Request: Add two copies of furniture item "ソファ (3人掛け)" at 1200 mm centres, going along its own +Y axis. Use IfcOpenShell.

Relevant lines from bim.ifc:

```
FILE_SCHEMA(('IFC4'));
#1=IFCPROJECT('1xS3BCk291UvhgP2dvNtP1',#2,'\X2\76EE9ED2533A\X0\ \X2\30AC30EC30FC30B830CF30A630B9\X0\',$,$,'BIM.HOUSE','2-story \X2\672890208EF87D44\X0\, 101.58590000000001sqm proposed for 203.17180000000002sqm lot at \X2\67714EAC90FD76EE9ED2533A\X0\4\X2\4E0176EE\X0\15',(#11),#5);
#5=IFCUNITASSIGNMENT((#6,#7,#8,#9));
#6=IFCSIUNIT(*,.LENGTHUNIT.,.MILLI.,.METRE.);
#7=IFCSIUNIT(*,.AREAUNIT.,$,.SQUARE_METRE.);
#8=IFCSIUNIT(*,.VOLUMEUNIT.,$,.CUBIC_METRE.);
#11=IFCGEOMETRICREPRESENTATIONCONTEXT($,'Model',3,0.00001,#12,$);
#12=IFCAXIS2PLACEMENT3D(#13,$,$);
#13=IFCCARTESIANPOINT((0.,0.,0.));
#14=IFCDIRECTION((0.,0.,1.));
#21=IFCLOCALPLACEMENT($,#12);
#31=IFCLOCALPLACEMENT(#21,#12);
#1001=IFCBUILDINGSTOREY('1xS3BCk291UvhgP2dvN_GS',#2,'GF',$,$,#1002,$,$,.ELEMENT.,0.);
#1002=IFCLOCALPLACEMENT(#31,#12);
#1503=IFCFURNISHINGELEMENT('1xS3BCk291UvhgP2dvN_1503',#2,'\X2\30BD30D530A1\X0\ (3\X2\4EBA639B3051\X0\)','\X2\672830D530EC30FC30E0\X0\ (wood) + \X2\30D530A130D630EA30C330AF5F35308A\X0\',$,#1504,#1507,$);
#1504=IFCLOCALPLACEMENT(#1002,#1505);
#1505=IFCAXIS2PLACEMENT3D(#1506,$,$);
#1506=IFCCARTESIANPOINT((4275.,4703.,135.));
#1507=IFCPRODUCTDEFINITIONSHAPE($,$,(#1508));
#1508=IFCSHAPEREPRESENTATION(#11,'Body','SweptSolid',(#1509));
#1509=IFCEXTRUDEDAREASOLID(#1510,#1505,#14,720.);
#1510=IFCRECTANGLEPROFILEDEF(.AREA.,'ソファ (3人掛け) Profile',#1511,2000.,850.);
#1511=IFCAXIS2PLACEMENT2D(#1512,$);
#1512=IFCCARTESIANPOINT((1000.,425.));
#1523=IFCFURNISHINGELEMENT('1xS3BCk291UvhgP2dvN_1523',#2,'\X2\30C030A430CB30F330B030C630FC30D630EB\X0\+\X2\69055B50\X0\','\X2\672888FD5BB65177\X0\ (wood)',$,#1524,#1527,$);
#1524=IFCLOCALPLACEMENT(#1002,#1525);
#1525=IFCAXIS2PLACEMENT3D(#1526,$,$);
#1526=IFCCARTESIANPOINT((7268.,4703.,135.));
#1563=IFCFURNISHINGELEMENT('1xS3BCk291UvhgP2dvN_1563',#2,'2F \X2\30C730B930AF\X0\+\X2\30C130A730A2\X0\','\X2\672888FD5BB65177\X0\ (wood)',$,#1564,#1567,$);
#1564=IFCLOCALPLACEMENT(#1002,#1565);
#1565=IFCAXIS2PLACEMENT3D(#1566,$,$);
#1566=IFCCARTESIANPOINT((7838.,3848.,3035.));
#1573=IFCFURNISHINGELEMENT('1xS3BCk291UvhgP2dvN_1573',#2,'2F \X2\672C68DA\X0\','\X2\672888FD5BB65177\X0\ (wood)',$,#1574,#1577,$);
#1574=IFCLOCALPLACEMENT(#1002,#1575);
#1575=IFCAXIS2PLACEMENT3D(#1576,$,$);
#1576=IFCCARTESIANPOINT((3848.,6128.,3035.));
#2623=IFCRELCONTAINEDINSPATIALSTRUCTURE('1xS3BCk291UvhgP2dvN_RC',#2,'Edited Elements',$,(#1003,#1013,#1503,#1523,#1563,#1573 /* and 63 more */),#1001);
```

```python
import ifcopenshell
import ifcopenshell.api.geometry
import ifcopenshell.api.root
import ifcopenshell.util.element
import ifcopenshell.util.placement

model = ifcopenshell.open("bim.ifc")


def reuse_history(source, copy):
    """copy_class also copies each property set's owner history, people and application; keep the originals."""
    for rel in copy.IsDefinedBy:
        if rel.is_a("IfcRelDefinesByProperties") and (history := rel.RelatingPropertyDefinition.OwnerHistory):
            rel.RelatingPropertyDefinition.OwnerHistory = source.OwnerHistory
            ifcopenshell.util.element.remove_deep2(model, history)


source = model.by_guid("1xS3BCk291UvhgP2dvN_1503")
base = ifcopenshell.util.placement.get_local_placement(source.ObjectPlacement)
step = base[:3, 1] * 1200.0

for i in range(1, 3):
    copy = ifcopenshell.api.root.copy_class(model, product=source)
    copy.Representation = ifcopenshell.util.element.copy_deep(
        model, source.Representation, exclude=["IfcGeometricRepresentationContext", "IfcRepresentationMap"]
    )
    reuse_history(source, copy)
    matrix = base.copy()
    matrix[:3, 3] += i * step
    print("added at", matrix[:3, 3].round(3) + 0.0)
    ifcopenshell.api.geometry.edit_object_placement(model, product=copy, matrix=matrix, is_si=False)

model.write("bim_v2.ifc")
```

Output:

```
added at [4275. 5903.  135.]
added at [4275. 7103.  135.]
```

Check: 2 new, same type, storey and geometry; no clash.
